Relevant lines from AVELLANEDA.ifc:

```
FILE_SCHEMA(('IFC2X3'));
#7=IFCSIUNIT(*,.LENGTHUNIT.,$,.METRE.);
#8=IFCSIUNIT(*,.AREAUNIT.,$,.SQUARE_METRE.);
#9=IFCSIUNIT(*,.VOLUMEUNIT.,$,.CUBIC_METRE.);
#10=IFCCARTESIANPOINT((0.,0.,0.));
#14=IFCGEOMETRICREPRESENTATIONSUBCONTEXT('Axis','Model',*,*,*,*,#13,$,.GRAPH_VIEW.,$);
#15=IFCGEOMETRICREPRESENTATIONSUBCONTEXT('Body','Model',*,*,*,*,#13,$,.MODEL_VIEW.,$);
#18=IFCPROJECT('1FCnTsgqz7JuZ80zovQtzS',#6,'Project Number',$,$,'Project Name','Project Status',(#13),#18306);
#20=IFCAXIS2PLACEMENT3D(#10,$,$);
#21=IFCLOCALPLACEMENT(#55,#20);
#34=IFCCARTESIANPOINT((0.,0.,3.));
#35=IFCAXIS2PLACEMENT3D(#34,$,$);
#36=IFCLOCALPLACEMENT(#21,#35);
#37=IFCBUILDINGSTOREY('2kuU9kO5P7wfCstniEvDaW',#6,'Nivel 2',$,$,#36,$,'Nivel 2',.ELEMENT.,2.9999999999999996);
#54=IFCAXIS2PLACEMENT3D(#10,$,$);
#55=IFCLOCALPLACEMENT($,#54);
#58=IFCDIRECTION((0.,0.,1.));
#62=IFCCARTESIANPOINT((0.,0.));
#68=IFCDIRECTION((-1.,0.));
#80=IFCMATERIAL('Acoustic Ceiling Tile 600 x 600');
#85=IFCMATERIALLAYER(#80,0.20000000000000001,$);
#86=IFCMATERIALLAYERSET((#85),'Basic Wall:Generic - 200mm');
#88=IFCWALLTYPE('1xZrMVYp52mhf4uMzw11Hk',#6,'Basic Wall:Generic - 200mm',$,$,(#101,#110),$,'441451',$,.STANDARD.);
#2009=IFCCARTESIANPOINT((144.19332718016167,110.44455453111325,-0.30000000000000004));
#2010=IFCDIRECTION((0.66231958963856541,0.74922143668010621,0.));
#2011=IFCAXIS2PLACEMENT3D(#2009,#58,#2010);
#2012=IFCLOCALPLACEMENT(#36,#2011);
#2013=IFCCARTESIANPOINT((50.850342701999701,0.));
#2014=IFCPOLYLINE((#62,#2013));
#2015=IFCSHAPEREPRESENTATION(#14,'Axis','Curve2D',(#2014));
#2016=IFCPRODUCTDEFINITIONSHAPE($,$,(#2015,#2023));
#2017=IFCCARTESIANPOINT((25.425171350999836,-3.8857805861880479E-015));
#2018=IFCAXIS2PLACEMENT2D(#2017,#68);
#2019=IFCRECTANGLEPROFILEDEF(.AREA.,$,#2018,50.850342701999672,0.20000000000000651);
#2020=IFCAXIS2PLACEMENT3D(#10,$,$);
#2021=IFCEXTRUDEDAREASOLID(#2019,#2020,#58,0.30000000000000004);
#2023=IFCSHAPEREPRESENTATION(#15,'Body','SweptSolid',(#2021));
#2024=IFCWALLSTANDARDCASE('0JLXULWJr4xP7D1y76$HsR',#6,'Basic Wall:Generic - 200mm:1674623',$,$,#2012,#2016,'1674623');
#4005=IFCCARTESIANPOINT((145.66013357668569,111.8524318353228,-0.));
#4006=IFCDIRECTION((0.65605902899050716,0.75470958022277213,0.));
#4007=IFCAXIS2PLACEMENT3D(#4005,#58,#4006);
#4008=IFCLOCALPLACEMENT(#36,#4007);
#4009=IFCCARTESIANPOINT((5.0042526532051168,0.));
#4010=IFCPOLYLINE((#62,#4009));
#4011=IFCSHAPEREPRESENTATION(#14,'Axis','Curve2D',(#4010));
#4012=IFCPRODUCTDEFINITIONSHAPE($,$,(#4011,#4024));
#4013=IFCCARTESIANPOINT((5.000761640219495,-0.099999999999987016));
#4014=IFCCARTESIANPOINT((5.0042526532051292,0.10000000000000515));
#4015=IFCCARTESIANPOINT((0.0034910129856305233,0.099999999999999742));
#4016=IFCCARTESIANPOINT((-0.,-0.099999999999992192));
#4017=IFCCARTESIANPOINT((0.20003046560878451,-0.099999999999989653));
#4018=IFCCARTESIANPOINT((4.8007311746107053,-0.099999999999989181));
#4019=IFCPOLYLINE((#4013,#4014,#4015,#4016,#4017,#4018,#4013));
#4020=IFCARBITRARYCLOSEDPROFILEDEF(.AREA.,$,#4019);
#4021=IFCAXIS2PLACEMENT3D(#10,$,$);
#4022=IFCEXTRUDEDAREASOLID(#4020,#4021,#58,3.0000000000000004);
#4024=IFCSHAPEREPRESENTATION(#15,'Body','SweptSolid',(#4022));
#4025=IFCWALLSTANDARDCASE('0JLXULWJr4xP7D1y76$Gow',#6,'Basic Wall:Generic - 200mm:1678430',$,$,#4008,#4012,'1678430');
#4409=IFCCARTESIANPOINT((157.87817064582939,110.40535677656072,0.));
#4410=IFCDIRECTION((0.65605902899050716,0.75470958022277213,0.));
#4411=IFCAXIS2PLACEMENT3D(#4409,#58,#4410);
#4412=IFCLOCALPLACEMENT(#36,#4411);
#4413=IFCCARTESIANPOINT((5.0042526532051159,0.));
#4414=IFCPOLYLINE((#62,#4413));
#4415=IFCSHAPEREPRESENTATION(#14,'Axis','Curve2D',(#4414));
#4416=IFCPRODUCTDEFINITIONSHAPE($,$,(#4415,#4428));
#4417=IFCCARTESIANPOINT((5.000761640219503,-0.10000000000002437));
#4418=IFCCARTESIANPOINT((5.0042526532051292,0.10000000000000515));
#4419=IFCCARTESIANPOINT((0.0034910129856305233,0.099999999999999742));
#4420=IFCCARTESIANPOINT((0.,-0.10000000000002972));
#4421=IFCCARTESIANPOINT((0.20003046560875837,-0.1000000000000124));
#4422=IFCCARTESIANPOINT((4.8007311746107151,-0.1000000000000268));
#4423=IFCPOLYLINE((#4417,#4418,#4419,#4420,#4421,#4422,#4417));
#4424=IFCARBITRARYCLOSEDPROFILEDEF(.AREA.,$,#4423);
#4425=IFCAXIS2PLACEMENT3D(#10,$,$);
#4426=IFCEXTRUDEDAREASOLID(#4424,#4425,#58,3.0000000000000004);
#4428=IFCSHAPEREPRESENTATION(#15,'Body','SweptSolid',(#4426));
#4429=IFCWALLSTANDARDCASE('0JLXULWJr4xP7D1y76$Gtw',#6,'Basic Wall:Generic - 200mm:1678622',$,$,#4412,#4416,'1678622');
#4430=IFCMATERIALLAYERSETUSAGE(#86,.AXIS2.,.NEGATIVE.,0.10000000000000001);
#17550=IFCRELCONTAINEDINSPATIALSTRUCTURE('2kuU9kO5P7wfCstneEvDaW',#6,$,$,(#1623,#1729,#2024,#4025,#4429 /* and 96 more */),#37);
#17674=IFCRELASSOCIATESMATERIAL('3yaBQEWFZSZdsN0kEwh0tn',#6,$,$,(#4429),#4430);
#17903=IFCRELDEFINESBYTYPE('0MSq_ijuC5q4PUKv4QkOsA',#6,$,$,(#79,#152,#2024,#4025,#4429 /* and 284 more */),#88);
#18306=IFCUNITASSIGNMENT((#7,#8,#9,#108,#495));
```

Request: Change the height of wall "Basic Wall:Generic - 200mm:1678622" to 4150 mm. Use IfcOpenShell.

```python
import ifcopenshell
import ifcopenshell.geom
import ifcopenshell.util.representation
import ifcopenshell.util.shape
import ifcopenshell.util.unit

model = ifcopenshell.open("AVELLANEDA.ifc")
unit_scale = ifcopenshell.util.unit.calculate_unit_scale(model)
settings = ifcopenshell.geom.settings()


def volume(element):
    """Net volume in cubic metres, openings subtracted."""
    shape = ifcopenshell.geom.create_shape(settings, element)
    return ifcopenshell.util.shape.get_volume(shape.geometry)


wall = model.by_guid("0JLXULWJr4xP7D1y76$Gtw")
before = volume(wall)

body = ifcopenshell.util.representation.get_representation(wall, "Model", "Body")
solid = body.Items[0]
old_height = solid.Depth
solid.Depth = 4.15 / unit_scale
after = volume(wall)

print(f"height {old_height:g} -> {solid.Depth:g}, volume {before:.3f} -> {after:.3f} m3")

model.write("AVELLANEDA_edited.ifc")
```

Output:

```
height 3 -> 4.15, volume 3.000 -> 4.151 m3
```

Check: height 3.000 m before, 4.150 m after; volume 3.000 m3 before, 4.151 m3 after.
